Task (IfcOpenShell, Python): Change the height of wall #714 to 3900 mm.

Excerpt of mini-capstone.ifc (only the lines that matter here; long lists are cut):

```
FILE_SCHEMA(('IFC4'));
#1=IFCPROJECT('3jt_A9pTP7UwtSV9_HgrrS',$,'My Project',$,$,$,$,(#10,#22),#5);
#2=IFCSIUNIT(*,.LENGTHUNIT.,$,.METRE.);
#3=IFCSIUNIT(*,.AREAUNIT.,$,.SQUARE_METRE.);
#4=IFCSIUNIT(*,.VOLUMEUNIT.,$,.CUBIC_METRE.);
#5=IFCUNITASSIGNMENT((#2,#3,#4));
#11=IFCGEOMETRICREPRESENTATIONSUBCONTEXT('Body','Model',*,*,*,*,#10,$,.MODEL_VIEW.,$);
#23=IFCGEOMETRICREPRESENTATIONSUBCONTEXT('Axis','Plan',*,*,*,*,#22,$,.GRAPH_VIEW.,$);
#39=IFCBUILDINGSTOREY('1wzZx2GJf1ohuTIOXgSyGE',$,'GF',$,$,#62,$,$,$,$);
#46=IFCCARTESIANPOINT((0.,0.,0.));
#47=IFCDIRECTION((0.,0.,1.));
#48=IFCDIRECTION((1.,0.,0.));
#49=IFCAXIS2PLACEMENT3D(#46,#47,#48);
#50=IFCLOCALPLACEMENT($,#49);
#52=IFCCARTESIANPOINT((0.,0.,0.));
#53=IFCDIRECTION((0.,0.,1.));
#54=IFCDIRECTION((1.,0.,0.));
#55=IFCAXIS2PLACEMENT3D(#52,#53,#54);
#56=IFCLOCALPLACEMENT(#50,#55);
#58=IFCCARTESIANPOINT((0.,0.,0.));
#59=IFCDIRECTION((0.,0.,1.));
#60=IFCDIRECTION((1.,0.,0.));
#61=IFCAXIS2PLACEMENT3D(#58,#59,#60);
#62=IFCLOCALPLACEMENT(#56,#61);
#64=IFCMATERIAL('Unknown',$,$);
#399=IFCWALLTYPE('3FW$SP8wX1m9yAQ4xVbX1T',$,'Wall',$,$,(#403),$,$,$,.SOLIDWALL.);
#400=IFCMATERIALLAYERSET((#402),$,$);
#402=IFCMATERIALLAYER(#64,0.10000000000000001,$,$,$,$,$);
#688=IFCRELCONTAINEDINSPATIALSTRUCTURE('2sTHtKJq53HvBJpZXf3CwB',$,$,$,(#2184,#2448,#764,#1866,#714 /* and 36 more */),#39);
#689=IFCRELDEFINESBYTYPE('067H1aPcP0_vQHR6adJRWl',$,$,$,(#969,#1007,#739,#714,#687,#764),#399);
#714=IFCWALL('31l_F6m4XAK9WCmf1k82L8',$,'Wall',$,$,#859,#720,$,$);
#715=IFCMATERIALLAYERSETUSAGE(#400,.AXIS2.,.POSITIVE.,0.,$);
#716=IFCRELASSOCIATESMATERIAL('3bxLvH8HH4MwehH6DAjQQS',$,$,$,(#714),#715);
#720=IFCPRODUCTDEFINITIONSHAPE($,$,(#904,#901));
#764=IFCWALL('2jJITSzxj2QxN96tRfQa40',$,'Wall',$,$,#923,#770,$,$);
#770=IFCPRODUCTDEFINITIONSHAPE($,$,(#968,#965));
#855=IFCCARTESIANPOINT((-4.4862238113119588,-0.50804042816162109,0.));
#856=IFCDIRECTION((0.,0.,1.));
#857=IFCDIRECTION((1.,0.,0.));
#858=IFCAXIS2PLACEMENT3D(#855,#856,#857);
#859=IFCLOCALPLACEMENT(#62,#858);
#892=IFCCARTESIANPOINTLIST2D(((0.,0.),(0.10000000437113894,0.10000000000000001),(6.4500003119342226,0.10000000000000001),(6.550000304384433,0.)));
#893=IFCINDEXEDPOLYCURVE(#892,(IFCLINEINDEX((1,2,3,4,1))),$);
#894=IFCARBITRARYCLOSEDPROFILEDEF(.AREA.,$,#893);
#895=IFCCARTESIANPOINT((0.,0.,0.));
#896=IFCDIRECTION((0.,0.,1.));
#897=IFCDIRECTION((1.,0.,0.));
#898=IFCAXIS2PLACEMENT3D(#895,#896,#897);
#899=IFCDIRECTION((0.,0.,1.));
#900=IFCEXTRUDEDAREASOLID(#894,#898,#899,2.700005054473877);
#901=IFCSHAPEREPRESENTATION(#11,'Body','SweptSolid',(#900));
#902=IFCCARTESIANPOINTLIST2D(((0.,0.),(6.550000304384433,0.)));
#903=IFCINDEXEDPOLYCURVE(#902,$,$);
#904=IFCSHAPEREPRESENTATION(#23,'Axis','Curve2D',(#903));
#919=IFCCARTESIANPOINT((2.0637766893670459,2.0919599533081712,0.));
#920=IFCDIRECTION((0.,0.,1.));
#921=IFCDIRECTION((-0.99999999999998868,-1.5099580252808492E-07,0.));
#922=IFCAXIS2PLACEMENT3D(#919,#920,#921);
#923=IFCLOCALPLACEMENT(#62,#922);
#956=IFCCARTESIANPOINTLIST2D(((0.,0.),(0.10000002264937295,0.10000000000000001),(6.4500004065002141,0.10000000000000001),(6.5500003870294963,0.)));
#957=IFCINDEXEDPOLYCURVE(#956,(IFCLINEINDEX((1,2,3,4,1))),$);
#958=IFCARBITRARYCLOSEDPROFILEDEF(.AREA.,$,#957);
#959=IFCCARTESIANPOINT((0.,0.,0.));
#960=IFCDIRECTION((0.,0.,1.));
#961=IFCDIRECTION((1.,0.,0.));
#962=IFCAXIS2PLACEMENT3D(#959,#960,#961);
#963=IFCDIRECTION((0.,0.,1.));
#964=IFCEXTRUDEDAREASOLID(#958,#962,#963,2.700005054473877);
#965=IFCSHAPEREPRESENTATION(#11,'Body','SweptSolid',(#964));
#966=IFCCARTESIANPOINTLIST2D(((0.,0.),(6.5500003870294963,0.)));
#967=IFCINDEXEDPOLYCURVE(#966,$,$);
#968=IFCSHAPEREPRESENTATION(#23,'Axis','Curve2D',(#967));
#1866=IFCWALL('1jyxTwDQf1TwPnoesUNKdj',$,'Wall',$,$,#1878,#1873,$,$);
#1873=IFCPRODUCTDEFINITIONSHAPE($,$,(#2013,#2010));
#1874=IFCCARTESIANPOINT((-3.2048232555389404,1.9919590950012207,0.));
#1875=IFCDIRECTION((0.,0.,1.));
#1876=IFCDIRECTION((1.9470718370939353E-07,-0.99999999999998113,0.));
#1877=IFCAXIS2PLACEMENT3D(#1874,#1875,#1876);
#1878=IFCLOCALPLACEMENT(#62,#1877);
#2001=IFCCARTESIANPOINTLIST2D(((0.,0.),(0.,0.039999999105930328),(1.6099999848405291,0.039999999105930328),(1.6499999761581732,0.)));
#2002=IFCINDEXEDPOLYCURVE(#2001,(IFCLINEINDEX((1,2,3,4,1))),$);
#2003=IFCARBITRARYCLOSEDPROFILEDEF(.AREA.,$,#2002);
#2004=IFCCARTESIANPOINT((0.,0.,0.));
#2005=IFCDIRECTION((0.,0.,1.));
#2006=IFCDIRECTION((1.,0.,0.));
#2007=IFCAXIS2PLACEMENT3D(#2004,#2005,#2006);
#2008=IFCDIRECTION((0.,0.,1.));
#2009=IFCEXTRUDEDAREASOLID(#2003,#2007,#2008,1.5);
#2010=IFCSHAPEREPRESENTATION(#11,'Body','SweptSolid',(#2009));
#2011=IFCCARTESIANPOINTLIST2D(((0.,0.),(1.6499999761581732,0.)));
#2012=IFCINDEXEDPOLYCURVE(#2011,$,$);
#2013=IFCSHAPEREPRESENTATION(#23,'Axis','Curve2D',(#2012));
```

```python
import ifcopenshell
import ifcopenshell.geom
import ifcopenshell.util.representation
import ifcopenshell.util.shape

model = ifcopenshell.open("mini-capstone.ifc")
settings = ifcopenshell.geom.settings()


def volume(element):
    """Net volume in cubic metres, openings subtracted."""
    shape = ifcopenshell.geom.create_shape(settings, element)
    return ifcopenshell.util.shape.get_volume(shape.geometry)


wall = model.by_id(714)
before = volume(wall)

body = ifcopenshell.util.representation.get_representation(wall, "Model", "Body")
solid = body.Items[0]
old_height = solid.Depth
solid.Depth = 3.9
after = volume(wall)

print(f"height {old_height:g} -> {solid.Depth:g}, volume {before:.3f} -> {after:.3f} m3")

model.write("mini-capstone_edited.ifc")
```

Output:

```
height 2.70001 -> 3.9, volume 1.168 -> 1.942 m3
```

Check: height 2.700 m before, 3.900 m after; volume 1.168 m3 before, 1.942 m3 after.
